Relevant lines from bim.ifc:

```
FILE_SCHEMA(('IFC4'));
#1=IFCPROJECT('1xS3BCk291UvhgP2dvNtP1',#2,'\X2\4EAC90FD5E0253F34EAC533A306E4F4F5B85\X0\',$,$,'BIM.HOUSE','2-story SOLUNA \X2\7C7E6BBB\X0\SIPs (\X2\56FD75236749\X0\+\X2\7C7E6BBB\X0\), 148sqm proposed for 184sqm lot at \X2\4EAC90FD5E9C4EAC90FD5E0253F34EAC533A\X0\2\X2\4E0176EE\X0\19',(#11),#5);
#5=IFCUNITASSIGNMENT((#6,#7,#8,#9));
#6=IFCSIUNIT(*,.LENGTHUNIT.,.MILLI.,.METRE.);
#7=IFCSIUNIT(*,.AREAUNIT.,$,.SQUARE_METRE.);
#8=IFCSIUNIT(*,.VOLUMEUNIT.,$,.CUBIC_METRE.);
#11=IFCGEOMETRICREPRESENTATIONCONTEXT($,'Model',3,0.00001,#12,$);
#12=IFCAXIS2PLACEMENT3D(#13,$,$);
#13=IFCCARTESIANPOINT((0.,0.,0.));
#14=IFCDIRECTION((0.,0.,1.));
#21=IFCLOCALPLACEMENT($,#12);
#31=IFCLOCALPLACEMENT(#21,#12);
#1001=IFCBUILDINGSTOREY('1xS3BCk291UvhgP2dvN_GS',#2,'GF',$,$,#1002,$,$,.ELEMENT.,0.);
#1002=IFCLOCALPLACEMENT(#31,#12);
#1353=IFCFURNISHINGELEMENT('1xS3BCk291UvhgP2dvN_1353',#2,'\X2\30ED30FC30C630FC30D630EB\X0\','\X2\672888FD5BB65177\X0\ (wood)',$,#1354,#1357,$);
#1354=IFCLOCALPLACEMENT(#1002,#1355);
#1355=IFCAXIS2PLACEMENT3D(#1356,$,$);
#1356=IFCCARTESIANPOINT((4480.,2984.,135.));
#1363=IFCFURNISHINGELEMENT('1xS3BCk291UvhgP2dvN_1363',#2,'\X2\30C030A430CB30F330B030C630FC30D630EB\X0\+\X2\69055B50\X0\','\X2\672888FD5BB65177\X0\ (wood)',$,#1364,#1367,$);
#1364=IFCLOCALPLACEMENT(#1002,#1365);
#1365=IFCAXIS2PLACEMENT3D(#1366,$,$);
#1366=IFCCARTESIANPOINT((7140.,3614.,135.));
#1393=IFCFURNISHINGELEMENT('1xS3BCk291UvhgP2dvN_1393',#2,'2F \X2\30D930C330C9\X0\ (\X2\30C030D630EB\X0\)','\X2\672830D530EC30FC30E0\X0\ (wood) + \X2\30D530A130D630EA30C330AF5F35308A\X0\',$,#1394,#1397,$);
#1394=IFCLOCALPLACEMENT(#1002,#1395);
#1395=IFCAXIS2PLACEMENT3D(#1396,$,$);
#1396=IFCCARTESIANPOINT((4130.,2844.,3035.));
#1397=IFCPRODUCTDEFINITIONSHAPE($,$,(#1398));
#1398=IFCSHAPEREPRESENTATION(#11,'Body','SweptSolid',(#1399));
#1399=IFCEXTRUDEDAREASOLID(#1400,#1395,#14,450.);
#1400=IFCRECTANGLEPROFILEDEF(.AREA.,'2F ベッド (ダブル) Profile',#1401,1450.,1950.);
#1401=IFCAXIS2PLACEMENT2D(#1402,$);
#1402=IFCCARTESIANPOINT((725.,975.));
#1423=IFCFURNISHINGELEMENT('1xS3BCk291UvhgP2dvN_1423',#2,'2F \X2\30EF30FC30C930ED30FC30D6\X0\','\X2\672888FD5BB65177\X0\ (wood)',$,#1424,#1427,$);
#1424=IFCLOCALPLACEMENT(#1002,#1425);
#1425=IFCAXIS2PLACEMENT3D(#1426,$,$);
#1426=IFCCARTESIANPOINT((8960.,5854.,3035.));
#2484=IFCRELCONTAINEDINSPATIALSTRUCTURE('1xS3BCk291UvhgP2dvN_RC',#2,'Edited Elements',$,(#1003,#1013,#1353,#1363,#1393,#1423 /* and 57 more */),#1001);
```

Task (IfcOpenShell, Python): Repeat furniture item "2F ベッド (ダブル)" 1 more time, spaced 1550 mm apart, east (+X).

```python
import numpy as np
import ifcopenshell
import ifcopenshell.api.geometry
import ifcopenshell.api.root
import ifcopenshell.util.element
import ifcopenshell.util.placement

model = ifcopenshell.open("bim.ifc")


def reuse_history(source, copy):
    """copy_class also copies each property set's owner history, people and application; keep the originals."""
    for rel in copy.IsDefinedBy:
        if rel.is_a("IfcRelDefinesByProperties") and (history := rel.RelatingPropertyDefinition.OwnerHistory):
            rel.RelatingPropertyDefinition.OwnerHistory = source.OwnerHistory
            ifcopenshell.util.element.remove_deep2(model, history)


source = model.by_guid("1xS3BCk291UvhgP2dvN_1393")
base = ifcopenshell.util.placement.get_local_placement(source.ObjectPlacement)
step = np.array([1.0, 0.0, 0.0]) * 1550.0

for i in range(1, 2):
    copy = ifcopenshell.api.root.copy_class(model, product=source)
    copy.Representation = ifcopenshell.util.element.copy_deep(
        model, source.Representation, exclude=["IfcGeometricRepresentationContext", "IfcRepresentationMap"]
    )
    reuse_history(source, copy)
    matrix = base.copy()
    matrix[:3, 3] += i * step
    print("added at", matrix[:3, 3].round(3) + 0.0)
    ifcopenshell.api.geometry.edit_object_placement(model, product=copy, matrix=matrix, is_si=False)

model.write("bim_rev.ifc")
```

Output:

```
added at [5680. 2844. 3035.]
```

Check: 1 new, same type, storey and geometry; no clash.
